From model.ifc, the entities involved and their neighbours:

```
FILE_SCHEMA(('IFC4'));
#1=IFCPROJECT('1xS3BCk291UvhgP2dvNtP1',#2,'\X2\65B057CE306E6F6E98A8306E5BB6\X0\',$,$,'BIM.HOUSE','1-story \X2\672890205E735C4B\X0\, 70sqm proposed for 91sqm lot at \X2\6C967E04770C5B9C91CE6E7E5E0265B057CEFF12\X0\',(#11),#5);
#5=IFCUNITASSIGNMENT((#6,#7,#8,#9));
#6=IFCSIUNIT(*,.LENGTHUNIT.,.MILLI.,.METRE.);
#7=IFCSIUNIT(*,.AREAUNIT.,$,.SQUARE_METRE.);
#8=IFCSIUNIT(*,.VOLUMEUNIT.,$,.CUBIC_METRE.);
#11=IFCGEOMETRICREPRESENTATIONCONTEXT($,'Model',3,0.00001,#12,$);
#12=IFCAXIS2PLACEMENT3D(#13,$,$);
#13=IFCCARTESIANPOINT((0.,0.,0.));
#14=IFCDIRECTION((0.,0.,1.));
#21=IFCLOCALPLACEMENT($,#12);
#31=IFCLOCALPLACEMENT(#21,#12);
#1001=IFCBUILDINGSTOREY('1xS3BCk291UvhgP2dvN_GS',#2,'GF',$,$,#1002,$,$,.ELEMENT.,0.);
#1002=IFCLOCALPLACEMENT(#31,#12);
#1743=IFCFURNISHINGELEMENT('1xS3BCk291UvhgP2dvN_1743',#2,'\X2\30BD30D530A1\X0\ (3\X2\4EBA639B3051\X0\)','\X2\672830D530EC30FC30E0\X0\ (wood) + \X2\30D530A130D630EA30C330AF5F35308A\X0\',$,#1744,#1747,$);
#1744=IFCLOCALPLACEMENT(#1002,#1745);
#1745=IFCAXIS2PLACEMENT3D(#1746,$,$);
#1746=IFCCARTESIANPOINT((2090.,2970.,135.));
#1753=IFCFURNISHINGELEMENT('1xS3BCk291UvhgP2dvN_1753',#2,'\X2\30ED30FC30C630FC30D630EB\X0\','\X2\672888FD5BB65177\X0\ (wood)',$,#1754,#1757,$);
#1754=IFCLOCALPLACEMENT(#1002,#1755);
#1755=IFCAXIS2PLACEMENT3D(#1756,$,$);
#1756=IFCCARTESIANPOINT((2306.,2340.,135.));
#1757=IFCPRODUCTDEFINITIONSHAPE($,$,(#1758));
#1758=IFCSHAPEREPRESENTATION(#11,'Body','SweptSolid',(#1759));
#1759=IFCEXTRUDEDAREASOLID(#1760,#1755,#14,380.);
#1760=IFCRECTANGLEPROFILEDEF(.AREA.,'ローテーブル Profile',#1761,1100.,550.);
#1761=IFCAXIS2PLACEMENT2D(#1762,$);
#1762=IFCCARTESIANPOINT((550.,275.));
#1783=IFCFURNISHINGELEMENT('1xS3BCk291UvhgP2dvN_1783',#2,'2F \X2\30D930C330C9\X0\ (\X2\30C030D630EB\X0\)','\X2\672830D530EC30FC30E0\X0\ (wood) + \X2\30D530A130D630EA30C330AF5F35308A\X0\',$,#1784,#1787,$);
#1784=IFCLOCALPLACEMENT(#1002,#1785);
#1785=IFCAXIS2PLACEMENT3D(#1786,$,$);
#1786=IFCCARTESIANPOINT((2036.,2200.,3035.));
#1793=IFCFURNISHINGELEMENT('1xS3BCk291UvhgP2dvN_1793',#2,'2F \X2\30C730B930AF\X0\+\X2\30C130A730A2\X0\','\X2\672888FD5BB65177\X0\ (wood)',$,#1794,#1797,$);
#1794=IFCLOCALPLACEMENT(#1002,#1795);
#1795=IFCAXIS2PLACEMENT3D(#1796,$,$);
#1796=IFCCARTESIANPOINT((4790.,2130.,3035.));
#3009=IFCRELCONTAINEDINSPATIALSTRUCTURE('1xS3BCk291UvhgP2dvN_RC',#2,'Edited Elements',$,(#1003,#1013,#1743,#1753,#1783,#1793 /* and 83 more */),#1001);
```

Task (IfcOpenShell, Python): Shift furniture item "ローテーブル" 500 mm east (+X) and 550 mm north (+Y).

```python
import ifcopenshell
import ifcopenshell.api.geometry
import ifcopenshell.util.placement

model = ifcopenshell.open("model.ifc")

item = model.by_guid("1xS3BCk291UvhgP2dvN_1753")
matrix = ifcopenshell.util.placement.get_local_placement(item.ObjectPlacement)
matrix[0, 3] += 500.0
matrix[1, 3] += 550.0
ifcopenshell.api.geometry.edit_object_placement(model, product=item, matrix=matrix, is_si=False)

print(ifcopenshell.util.placement.get_local_placement(item.ObjectPlacement).round(3) + 0.0)

model.write("model_v2.ifc")
```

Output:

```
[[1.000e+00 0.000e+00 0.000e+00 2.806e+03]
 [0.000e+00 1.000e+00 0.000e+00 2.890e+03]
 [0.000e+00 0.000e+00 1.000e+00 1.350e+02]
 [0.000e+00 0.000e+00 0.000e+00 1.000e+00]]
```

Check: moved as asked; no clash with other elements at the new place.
